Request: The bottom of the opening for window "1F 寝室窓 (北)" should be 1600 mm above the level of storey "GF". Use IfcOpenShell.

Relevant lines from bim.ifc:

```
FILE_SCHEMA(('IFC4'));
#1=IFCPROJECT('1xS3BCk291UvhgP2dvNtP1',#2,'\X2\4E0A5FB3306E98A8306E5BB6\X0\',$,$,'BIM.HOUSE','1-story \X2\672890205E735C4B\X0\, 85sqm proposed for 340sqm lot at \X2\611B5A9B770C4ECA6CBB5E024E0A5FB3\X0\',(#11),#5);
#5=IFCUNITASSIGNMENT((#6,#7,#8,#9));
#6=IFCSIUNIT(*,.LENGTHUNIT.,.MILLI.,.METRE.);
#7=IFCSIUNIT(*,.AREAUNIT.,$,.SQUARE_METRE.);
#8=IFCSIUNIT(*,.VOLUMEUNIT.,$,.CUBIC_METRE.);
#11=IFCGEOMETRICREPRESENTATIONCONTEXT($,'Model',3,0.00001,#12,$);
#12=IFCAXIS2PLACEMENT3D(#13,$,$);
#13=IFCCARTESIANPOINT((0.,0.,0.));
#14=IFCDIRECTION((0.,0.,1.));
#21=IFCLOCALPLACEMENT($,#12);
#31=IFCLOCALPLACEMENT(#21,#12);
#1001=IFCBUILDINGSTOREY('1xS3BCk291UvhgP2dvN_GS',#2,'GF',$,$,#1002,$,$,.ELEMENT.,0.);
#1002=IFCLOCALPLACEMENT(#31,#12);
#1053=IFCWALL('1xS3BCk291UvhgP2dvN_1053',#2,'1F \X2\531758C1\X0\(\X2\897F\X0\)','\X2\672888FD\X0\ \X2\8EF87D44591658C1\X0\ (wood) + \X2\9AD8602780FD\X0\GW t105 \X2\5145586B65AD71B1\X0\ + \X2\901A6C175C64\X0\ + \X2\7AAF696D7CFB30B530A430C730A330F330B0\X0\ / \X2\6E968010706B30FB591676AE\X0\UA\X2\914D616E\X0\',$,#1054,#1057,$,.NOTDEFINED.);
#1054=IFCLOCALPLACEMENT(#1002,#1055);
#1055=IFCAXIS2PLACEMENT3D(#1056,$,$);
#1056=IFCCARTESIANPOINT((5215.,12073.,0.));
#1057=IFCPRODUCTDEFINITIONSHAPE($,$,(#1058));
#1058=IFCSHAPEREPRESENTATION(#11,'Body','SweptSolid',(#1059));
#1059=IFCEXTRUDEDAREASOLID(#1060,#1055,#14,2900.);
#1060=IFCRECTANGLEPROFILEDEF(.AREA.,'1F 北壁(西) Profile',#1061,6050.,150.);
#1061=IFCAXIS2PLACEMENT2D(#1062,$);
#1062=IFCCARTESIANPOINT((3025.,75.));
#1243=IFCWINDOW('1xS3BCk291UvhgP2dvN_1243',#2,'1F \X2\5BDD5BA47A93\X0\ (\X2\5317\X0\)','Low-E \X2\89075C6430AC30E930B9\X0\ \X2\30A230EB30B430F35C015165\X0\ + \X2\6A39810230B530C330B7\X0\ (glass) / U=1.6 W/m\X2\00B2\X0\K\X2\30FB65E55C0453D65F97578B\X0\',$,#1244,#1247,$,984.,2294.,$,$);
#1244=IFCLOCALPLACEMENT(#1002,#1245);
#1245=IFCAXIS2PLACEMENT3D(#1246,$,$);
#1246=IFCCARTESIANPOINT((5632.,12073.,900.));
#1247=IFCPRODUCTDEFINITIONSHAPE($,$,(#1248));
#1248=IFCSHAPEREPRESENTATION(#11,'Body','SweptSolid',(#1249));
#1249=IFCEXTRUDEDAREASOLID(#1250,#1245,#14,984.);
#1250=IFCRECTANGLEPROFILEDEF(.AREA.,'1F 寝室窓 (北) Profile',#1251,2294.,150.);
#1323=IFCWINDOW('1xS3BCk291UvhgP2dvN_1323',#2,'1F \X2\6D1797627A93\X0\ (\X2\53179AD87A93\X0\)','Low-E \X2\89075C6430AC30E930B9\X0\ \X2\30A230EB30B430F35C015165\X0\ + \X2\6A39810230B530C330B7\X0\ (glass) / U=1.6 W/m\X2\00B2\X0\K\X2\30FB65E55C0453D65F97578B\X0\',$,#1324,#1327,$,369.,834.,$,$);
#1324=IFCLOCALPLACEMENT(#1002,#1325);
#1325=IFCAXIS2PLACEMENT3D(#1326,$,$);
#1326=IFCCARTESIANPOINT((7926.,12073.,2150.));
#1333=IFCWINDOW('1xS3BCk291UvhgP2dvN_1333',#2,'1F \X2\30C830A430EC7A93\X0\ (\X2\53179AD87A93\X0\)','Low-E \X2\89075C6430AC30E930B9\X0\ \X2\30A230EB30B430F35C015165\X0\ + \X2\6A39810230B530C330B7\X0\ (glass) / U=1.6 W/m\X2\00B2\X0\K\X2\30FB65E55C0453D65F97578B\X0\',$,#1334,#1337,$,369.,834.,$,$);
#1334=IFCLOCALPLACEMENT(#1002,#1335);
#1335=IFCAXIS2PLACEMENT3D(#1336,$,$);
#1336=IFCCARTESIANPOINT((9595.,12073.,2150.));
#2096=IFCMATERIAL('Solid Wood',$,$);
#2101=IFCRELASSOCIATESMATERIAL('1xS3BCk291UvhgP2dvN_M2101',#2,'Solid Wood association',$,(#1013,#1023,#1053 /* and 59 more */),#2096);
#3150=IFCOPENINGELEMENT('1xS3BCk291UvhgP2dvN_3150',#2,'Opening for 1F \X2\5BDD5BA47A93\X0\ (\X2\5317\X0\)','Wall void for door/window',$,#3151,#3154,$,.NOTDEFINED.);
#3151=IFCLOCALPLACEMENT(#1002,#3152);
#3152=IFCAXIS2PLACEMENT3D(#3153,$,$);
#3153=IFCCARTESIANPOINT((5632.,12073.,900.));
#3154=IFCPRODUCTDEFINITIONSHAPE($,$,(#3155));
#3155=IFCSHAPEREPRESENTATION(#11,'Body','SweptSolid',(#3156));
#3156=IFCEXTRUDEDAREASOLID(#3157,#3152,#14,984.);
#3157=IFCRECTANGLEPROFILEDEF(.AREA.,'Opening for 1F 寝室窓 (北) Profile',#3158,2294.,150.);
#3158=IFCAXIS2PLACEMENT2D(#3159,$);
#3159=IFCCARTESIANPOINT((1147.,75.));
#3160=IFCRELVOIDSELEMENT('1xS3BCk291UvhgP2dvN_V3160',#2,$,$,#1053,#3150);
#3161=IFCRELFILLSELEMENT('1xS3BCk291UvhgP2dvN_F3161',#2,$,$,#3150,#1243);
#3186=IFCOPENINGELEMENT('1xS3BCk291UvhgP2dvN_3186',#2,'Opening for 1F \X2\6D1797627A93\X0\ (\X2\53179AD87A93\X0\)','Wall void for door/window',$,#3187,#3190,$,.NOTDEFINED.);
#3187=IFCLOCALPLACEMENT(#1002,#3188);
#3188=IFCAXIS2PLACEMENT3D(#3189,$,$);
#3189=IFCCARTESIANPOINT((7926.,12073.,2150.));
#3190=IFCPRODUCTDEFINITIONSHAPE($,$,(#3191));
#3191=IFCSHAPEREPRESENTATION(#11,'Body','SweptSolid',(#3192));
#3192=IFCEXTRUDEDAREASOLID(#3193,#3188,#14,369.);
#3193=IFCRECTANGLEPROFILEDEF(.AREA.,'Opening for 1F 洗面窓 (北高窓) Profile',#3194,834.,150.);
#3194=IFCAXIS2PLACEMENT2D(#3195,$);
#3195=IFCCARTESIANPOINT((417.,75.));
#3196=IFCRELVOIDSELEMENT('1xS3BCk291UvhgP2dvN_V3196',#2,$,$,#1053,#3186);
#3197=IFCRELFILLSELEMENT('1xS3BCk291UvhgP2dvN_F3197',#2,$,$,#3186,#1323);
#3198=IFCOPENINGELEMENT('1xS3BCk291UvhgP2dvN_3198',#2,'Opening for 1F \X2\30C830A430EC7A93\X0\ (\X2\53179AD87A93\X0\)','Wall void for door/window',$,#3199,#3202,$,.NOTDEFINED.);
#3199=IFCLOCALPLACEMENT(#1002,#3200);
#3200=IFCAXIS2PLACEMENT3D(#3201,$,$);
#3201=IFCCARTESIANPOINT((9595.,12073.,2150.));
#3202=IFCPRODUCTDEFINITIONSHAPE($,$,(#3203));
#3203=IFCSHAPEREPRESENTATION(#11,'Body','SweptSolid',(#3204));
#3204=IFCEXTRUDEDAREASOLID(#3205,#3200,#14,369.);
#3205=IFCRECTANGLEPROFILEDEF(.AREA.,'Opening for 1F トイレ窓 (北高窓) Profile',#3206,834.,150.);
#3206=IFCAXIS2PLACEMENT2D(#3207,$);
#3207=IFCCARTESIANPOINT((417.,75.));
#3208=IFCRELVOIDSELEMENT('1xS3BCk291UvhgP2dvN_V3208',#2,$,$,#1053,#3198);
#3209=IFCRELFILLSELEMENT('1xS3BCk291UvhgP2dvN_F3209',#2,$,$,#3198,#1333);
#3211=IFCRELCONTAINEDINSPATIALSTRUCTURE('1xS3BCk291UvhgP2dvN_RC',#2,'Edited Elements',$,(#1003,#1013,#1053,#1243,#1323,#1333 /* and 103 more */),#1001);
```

```python
import numpy as np
import ifcopenshell
import ifcopenshell.api.geometry
import ifcopenshell.geom
import ifcopenshell.util.element
import ifcopenshell.util.placement
import ifcopenshell.util.shape
import ifcopenshell.util.unit

model = ifcopenshell.open("bim.ifc")
unit_scale = ifcopenshell.util.unit.calculate_unit_scale(model)

window = model.by_guid("1xS3BCk291UvhgP2dvN_1243")
opening = window.FillsVoids[0].RelatingOpeningElement
storey = ifcopenshell.util.element.get_container(window, ifc_class="IfcBuildingStorey")
level = ifcopenshell.util.placement.get_local_placement(storey.ObjectPlacement)[2, 3]

# The opening's origin need not be at the sill, so measure its lowest point.
shape = ifcopenshell.geom.create_shape(ifcopenshell.geom.settings(), opening)
bottom = ifcopenshell.util.shape.get_shape_bottom_elevation(shape, shape.geometry) / unit_scale
dz = level + 1600.0 - bottom

shift = np.array([0.0, 0.0, dz])
# The window is not placed relative to its opening, so move both.
for product in (opening, window):
    matrix = ifcopenshell.util.placement.get_local_placement(product.ObjectPlacement)
    matrix[:3, 3] += shift
    ifcopenshell.api.geometry.edit_object_placement(model, product=product, matrix=matrix, is_si=False)

print(f"moved by {dz * unit_scale:+.3f} m")

model.write("bim_rev.ifc")
```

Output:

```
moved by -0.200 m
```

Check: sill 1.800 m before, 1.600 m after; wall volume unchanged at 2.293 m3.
